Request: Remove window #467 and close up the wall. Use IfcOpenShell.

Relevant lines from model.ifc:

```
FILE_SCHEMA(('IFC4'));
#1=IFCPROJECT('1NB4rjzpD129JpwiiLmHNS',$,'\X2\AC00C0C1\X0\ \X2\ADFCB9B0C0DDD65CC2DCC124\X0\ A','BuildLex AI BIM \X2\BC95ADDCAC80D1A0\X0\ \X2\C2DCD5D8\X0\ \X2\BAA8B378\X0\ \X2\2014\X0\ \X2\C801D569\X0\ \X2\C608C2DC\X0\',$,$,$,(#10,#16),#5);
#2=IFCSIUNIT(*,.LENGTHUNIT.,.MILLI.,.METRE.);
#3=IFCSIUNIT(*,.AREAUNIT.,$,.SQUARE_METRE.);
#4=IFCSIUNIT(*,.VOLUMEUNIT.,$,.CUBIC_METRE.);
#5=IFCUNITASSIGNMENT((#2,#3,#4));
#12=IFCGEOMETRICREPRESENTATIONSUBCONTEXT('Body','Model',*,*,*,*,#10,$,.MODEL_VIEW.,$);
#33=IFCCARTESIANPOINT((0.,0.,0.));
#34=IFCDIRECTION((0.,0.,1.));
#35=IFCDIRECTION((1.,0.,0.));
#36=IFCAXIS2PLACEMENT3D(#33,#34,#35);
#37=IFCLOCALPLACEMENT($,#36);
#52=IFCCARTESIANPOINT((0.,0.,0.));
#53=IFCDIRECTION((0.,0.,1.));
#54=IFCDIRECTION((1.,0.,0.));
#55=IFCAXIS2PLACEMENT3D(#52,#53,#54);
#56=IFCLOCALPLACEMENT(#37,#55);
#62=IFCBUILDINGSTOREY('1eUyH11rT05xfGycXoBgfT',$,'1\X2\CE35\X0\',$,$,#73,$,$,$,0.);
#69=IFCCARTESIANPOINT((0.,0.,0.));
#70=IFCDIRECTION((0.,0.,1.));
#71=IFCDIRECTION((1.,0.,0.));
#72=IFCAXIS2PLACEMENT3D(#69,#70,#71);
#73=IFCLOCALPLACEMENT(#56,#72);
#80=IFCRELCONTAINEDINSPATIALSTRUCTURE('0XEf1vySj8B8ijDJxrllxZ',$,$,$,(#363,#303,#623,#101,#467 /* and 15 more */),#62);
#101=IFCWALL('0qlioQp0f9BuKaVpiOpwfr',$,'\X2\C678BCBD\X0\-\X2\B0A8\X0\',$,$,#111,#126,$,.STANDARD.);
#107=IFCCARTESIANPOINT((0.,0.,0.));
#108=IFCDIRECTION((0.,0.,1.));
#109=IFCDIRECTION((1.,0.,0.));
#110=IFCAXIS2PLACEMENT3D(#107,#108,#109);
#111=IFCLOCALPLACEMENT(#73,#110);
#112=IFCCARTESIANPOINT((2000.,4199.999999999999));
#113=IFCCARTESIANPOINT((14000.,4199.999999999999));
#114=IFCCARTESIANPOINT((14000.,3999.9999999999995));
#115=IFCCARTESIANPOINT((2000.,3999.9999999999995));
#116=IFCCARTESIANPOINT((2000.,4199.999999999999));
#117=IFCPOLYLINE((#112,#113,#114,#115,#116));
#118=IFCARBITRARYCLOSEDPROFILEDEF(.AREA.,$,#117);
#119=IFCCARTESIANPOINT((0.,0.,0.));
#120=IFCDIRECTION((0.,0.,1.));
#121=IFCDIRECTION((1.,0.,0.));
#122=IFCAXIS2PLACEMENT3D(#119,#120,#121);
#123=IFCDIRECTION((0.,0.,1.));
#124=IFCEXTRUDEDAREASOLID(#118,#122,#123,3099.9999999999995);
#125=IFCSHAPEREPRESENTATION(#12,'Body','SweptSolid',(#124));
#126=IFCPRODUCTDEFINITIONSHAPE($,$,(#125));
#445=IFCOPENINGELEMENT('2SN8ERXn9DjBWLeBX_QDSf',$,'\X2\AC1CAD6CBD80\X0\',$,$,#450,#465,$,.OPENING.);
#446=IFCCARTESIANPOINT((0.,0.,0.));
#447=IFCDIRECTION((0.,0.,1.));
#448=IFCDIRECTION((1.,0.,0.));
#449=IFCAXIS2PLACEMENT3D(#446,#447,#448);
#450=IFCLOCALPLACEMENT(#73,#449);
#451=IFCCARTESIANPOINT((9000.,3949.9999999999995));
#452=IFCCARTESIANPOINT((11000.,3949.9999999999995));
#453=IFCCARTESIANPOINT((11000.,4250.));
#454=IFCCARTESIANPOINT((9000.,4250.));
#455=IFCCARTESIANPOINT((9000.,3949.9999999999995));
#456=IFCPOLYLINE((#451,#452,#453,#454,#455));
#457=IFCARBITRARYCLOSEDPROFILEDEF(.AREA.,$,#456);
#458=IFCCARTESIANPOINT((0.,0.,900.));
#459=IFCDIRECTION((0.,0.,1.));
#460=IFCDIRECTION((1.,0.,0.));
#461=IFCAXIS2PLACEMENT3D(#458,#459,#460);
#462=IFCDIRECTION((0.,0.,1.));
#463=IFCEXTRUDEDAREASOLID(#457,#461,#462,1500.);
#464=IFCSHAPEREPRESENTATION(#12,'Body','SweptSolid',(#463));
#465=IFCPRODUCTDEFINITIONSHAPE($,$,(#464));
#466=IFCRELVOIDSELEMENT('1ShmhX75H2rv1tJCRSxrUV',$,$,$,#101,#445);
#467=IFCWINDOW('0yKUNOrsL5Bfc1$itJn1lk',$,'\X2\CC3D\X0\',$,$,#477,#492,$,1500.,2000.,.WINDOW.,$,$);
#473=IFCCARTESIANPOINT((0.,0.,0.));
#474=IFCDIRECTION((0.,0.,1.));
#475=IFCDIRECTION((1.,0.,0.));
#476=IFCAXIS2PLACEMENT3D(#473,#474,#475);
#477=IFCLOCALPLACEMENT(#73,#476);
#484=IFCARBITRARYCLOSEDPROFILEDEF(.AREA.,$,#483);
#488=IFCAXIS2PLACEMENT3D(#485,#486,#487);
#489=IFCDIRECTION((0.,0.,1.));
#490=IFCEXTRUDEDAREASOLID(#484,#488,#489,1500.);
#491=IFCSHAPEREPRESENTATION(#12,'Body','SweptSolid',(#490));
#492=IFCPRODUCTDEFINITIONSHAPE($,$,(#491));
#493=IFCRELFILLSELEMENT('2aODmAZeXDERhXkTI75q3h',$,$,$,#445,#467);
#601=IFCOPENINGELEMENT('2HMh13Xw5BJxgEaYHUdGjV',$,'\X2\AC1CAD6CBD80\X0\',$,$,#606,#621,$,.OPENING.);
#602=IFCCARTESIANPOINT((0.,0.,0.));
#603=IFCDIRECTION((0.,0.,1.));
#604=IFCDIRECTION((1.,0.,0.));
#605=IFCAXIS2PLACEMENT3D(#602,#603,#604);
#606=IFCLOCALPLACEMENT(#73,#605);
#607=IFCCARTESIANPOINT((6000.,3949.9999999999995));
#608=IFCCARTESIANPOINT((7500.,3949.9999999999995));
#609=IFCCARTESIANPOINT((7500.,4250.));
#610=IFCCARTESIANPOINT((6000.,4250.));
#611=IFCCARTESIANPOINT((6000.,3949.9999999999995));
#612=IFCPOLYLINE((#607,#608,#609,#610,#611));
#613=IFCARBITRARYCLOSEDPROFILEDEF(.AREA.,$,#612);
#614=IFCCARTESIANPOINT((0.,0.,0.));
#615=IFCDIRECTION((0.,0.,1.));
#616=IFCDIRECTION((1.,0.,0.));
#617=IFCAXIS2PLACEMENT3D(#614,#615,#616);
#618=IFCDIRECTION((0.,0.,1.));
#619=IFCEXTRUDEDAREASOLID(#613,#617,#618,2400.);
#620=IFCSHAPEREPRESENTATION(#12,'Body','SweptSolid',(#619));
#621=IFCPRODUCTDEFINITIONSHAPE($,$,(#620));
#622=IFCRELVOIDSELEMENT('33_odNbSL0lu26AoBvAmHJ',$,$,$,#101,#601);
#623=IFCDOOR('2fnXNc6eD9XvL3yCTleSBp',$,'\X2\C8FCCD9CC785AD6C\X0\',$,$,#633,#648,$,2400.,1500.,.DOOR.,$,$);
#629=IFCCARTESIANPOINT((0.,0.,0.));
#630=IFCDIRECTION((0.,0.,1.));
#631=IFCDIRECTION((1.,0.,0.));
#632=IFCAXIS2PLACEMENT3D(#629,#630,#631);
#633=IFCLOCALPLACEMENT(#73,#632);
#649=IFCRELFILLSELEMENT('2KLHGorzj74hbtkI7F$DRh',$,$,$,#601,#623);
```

```python
import ifcopenshell
import ifcopenshell.api.feature
import ifcopenshell.api.root
import ifcopenshell.geom
import ifcopenshell.util.shape

model = ifcopenshell.open("model.ifc")
settings = ifcopenshell.geom.settings()


def volume(element):
    """Net volume in cubic metres, openings subtracted."""
    shape = ifcopenshell.geom.create_shape(settings, element)
    return ifcopenshell.util.shape.get_volume(shape.geometry)


window = model.by_guid("0yKUNOrsL5Bfc1$itJn1lk")
opening = window.FillsVoids[0].RelatingOpeningElement
wall = opening.VoidsElements[0].RelatingBuildingElement
before = volume(wall)

ifcopenshell.api.root.remove_product(model, product=window)
ifcopenshell.api.feature.remove_feature(model, feature=opening)

after = volume(wall)

print(f"wall volume {before:.3f} -> {after:.3f} m3")

model.write("model_v2.ifc")
```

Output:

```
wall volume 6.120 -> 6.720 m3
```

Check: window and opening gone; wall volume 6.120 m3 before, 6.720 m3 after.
